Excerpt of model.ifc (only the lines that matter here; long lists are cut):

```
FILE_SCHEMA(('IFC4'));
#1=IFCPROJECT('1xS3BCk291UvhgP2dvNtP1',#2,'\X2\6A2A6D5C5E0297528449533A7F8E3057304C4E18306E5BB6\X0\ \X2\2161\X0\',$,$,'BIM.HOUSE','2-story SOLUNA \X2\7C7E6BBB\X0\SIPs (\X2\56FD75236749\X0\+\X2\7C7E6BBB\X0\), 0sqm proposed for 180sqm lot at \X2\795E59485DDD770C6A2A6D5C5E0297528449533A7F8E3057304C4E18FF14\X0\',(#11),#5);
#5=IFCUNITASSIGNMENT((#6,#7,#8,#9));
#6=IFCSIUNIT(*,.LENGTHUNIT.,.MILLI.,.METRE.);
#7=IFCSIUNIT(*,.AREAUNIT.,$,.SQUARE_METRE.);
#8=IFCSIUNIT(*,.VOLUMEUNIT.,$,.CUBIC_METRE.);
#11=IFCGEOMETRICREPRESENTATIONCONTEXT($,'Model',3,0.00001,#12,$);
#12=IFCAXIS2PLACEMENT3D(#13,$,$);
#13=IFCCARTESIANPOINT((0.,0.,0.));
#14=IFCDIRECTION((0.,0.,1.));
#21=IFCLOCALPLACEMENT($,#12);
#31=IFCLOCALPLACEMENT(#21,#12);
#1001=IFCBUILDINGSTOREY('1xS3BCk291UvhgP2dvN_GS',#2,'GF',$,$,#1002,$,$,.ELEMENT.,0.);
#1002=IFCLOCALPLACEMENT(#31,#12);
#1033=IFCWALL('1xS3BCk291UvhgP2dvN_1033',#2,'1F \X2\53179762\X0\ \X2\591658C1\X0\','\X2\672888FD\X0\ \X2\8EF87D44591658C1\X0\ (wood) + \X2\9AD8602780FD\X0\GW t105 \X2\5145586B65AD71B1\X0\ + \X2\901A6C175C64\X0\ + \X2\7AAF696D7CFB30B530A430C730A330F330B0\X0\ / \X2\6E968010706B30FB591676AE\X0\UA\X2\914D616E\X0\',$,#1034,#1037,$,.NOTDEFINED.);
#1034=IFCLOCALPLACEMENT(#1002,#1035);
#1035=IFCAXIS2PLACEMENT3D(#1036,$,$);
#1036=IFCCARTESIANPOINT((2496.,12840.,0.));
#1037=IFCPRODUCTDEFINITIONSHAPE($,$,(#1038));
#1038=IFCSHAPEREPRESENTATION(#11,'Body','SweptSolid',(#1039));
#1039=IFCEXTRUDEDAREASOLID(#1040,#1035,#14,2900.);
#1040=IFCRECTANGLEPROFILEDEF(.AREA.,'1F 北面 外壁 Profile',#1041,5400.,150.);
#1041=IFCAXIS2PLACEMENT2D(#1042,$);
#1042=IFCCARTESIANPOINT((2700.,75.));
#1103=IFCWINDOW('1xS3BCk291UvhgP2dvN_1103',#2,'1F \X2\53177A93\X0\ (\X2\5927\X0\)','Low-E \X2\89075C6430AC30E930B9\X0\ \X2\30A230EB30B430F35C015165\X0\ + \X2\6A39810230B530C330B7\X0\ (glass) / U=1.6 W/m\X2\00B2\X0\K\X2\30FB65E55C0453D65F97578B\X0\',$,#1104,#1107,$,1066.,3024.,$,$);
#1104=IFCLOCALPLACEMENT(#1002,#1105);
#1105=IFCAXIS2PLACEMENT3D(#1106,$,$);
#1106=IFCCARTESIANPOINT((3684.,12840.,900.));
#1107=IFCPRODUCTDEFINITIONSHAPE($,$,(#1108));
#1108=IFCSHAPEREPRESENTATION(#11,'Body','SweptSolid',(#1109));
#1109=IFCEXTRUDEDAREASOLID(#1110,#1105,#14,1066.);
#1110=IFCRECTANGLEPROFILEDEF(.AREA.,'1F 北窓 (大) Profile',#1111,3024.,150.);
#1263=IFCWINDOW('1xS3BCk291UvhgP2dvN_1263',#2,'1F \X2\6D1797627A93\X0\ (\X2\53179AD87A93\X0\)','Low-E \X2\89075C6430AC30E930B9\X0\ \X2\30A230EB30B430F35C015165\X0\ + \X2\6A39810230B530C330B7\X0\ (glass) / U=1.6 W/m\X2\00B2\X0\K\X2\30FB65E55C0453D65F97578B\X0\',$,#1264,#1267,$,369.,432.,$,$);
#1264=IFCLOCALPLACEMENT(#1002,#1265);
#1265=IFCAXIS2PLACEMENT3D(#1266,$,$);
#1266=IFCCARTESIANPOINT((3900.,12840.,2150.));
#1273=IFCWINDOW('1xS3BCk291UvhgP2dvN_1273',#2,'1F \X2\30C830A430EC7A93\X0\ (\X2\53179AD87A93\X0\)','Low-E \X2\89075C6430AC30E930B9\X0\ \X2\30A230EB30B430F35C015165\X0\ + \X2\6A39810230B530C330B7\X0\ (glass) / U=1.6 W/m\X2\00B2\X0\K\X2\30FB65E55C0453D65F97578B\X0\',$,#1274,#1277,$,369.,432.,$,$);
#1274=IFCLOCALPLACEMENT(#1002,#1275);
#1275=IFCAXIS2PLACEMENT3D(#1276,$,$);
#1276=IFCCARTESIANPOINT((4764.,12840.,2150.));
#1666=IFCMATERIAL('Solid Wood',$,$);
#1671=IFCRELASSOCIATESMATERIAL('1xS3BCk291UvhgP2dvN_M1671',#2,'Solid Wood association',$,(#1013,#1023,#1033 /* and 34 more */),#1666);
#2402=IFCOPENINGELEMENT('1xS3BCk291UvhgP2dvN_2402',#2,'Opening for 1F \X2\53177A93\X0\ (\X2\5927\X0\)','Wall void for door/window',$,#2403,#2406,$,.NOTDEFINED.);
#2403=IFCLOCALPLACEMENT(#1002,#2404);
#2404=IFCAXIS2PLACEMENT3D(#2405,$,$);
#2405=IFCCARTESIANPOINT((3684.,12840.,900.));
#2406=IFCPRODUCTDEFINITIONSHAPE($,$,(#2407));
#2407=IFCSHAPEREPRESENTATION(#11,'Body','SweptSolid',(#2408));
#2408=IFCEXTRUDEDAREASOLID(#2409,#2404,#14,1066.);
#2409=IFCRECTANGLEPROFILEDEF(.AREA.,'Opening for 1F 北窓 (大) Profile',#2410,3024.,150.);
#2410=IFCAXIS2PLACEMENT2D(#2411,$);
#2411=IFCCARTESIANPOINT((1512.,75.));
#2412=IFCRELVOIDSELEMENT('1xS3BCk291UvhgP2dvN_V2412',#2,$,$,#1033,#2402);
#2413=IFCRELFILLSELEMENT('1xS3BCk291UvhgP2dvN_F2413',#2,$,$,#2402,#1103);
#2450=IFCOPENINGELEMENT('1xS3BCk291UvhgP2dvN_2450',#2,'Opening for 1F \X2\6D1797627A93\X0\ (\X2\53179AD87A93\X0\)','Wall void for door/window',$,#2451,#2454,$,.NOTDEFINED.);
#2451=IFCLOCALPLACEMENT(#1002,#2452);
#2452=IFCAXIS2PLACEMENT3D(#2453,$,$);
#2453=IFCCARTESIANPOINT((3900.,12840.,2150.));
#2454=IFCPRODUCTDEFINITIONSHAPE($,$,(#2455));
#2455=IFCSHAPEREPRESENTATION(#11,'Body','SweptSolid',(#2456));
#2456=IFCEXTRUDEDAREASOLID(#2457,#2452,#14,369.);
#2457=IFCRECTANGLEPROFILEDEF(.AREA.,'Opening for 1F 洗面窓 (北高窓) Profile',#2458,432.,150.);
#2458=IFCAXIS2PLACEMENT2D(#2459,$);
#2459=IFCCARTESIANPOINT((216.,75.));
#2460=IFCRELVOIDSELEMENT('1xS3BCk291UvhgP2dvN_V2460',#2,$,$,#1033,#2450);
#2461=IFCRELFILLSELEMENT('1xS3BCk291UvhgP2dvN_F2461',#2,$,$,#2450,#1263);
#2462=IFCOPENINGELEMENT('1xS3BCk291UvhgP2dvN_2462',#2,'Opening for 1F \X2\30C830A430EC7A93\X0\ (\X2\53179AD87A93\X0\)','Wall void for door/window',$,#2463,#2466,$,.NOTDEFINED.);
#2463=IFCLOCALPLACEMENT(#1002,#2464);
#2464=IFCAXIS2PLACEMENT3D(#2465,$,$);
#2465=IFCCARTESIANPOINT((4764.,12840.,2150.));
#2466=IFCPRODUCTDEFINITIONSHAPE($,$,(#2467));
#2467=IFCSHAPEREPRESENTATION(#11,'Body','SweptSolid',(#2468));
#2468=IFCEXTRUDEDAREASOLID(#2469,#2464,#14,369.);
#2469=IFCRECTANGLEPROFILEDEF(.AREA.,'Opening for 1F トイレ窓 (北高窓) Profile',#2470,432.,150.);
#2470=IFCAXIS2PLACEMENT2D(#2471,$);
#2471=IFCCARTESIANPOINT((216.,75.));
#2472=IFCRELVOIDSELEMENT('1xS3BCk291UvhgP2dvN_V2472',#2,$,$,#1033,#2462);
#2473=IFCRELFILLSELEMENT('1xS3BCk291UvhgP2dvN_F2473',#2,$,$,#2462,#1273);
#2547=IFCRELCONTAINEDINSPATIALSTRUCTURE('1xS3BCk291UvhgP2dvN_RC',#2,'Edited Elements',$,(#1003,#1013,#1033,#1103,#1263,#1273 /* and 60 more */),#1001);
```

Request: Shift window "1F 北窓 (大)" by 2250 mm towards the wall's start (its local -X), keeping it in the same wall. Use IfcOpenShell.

```python
import ifcopenshell
import ifcopenshell.api.geometry
import ifcopenshell.util.placement

model = ifcopenshell.open("model.ifc")

window = model.by_guid("1xS3BCk291UvhgP2dvN_1103")
opening = window.FillsVoids[0].RelatingOpeningElement
wall = opening.VoidsElements[0].RelatingBuildingElement

wall_matrix = ifcopenshell.util.placement.get_local_placement(wall.ObjectPlacement)
shift = wall_matrix[:3, 0] * -2250.0
before = ifcopenshell.util.placement.get_local_placement(window.ObjectPlacement)[:3, 3].copy()

# The window is not placed relative to its opening, so move both.
for product in (opening, window):
    matrix = ifcopenshell.util.placement.get_local_placement(product.ObjectPlacement)
    matrix[:3, 3] += shift
    ifcopenshell.api.geometry.edit_object_placement(model, product=product, matrix=matrix, is_si=False)

after = ifcopenshell.util.placement.get_local_placement(window.ObjectPlacement)[:3, 3]
print("window moved by", (after - before).round(3) + 0.0)

model.write("model-out.ifc")
```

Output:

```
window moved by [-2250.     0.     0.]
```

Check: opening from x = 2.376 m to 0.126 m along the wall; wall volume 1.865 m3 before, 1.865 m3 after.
